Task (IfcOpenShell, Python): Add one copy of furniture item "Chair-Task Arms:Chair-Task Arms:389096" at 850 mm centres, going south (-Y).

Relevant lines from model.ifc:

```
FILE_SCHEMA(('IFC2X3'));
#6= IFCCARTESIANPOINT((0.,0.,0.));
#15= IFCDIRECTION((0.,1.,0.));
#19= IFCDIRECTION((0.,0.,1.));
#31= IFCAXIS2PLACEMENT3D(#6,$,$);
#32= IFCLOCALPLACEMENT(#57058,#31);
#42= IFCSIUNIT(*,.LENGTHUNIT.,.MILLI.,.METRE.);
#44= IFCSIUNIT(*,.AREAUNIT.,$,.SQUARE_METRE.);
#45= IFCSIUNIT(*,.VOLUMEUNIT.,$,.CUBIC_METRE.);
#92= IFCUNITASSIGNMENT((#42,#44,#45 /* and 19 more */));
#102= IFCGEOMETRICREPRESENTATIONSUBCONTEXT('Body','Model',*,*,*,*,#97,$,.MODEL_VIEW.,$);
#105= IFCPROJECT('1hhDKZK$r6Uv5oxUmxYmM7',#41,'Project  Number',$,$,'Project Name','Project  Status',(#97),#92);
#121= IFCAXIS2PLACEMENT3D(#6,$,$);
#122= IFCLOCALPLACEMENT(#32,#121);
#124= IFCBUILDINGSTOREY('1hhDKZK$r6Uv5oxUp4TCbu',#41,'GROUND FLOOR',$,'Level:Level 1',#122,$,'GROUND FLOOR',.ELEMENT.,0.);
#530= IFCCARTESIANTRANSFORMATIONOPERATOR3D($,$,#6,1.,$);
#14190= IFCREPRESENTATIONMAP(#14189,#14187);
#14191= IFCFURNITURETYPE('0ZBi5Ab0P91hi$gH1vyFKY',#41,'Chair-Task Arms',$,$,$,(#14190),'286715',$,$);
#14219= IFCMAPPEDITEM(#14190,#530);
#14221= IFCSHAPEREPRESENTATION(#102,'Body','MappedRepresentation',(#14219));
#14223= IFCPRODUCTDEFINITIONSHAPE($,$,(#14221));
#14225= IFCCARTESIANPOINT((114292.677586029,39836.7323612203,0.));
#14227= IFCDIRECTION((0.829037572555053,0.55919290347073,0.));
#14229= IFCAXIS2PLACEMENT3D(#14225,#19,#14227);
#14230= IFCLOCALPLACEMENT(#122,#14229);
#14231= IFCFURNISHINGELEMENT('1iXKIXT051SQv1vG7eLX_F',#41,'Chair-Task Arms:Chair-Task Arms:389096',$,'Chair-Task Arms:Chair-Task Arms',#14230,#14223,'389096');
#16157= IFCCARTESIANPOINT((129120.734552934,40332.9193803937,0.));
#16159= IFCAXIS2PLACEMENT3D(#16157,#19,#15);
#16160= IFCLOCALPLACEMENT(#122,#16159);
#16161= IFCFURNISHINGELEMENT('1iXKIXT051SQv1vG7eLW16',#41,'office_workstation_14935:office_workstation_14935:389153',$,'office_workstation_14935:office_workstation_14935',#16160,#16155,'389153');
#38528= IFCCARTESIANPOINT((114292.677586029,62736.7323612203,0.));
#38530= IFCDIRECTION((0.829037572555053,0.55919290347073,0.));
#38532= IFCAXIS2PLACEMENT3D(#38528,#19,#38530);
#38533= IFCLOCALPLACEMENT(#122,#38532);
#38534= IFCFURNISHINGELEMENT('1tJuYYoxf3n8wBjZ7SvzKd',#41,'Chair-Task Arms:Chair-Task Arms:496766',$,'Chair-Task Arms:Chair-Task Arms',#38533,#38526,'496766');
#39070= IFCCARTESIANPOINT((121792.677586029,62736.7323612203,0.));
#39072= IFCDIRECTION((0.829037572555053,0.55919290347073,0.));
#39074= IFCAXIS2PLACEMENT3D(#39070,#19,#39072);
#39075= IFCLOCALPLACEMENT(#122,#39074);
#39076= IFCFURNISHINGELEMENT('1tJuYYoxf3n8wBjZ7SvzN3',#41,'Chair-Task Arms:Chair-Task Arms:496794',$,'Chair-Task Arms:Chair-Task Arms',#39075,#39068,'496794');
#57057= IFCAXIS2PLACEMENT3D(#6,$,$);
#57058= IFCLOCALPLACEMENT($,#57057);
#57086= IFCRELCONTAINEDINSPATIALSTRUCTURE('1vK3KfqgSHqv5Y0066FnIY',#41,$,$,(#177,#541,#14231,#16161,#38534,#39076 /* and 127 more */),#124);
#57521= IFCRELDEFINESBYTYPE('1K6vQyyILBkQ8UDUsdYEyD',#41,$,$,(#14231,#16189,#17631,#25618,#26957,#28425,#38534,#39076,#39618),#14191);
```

```python
import numpy as np
import ifcopenshell
import ifcopenshell.api.geometry
import ifcopenshell.api.root
import ifcopenshell.util.element
import ifcopenshell.util.placement
import ifcopenshell.util.unit

model = ifcopenshell.open("model.ifc")
unit_scale = ifcopenshell.util.unit.calculate_unit_scale(model)


def reuse_history(source, copy):
    """copy_class also copies each property set's owner history, people and application; keep the originals."""
    for rel in copy.IsDefinedBy:
        if rel.is_a("IfcRelDefinesByProperties") and (history := rel.RelatingPropertyDefinition.OwnerHistory):
            rel.RelatingPropertyDefinition.OwnerHistory = source.OwnerHistory
            ifcopenshell.util.element.remove_deep2(model, history)


source = model.by_guid("1iXKIXT051SQv1vG7eLX_F")
base = ifcopenshell.util.placement.get_local_placement(source.ObjectPlacement)
step = np.array([0.0, -1.0, 0.0]) * 0.85 / unit_scale

for i in range(1, 2):
    copy = ifcopenshell.api.root.copy_class(model, product=source)
    copy.Representation = ifcopenshell.util.element.copy_deep(
        model, source.Representation, exclude=["IfcGeometricRepresentationContext", "IfcRepresentationMap"]
    )
    copy.Name = "Chair-Task Arms:Chair-Task Arms"
    copy.Tag = None
    reuse_history(source, copy)
    matrix = base.copy()
    matrix[:3, 3] += i * step
    print("added at", matrix[:3, 3].round(3) + 0.0)
    ifcopenshell.api.geometry.edit_object_placement(model, product=copy, matrix=matrix, is_si=False)

model.write("model_rev.ifc")
```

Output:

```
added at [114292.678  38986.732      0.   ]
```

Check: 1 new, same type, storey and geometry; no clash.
